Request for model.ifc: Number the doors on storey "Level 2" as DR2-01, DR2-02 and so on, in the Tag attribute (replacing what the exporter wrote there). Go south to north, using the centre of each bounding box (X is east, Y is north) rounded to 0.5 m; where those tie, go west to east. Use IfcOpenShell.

First a look at what the model holds.

```python
import ifcopenshell
import ifcopenshell.util.element
import ifcopenshell.util.placement

model = ifcopenshell.open("model.ifc")
print(model.schema)
storey = next(s for s in model.by_type("IfcBuildingStorey") if s.Name == "Level 2")
doors = [e for e in ifcopenshell.util.element.get_decomposition(storey) if e.is_a("IfcDoor")]
for e in sorted(doors, key=lambda e: e.id()):
    origin = ifcopenshell.util.placement.get_local_placement(e.ObjectPlacement)[:3, 3]
    print(e.id(), e.Tag, e.Name, origin.round(2) + 0.0, sep=" | ")
```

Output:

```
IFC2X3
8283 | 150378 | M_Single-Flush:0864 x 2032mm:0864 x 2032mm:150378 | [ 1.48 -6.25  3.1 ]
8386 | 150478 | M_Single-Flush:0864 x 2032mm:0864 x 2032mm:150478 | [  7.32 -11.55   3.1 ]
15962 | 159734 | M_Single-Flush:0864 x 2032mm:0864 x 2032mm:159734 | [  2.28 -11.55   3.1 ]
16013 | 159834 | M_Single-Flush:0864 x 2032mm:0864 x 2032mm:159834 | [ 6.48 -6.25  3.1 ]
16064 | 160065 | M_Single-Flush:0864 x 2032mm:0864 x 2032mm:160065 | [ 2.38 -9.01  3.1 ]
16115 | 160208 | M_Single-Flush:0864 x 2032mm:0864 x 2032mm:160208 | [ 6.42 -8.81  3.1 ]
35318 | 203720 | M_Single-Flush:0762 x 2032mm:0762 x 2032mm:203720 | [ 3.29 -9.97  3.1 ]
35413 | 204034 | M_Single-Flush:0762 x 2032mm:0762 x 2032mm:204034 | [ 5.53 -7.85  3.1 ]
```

```python
import ifcopenshell
import ifcopenshell.geom
import ifcopenshell.util.element
import ifcopenshell.util.shape

model = ifcopenshell.open("model.ifc")
settings = ifcopenshell.geom.settings()
settings.set("use-world-coords", True)


def centre(element):
    shape = ifcopenshell.geom.create_shape(settings, element)
    return ifcopenshell.util.shape.get_bbox_centroid(shape.geometry)


storey = next(s for s in model.by_type("IfcBuildingStorey") if s.Name == "Level 2")
doors = [e for e in ifcopenshell.util.element.get_decomposition(storey) if e.is_a("IfcDoor")]

# Insertion points can sit at a corner or the storey origin, so sort by the geometry (in metres).
centres = {e: centre(e) for e in doors}
doors.sort(key=lambda e: (round(centres[e][1] / 0.5), centres[e][0]))

for i, e in enumerate(doors, start=1):
    number = f"DR2-{i:02d}"
    e.Tag = number
    print(e.id(), number)

model.write("model-out.ifc")
```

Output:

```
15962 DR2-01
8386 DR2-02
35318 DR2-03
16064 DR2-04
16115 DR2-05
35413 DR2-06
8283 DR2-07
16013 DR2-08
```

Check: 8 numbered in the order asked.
